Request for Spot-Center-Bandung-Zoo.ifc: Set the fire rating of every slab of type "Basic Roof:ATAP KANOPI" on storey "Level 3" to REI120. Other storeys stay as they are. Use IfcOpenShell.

First a look at what the model holds.

```python
import ifcopenshell
import ifcopenshell.util.element

model = ifcopenshell.open("Spot-Center-Bandung-Zoo.ifc")
print(model.schema)
storey = next(s for s in model.by_type("IfcBuildingStorey") if s.Name == "Level 3")
slabs = [e for e in ifcopenshell.util.element.get_decomposition(storey) if e.is_a("IfcSlab")]
seen = {}
for e in slabs:
    element_type = ifcopenshell.util.element.get_type(e)
    key = (element_type.Name if element_type != e and element_type else None, ifcopenshell.util.element.get_pset(e, "Pset_SlabCommon", "FireRating"))
    seen[key] = seen.get(key, 0) + 1
for (name, value), count in sorted(seen.items(), key=str):
    print(count, "x", name, "|", value)
```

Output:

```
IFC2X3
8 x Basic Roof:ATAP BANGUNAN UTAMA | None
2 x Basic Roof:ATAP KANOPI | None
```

```python
import ifcopenshell
import ifcopenshell.api.pset
import ifcopenshell.util.element

model = ifcopenshell.open("Spot-Center-Bandung-Zoo.ifc")

storey = next(s for s in model.by_type("IfcBuildingStorey") if s.Name == "Level 3")
slabs = [e for e in ifcopenshell.util.element.get_decomposition(storey) if e.is_a("IfcSlab")]

count = 0
for e in slabs:
    element_type = ifcopenshell.util.element.get_type(e)
    if element_type in (None, e) or element_type.Name != "Basic Roof:ATAP KANOPI":
        continue
    # add_pset returns the element's existing set when there is one.
    pset = ifcopenshell.api.pset.add_pset(model, product=e, name="Pset_SlabCommon")
    ifcopenshell.api.pset.edit_pset(model, pset=pset, properties={"FireRating": "REI120"})
    count += 1

print(count, "slabs updated")

model.write("Spot-Center-Bandung-Zoo-out.ifc")
```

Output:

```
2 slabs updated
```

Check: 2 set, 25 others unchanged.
